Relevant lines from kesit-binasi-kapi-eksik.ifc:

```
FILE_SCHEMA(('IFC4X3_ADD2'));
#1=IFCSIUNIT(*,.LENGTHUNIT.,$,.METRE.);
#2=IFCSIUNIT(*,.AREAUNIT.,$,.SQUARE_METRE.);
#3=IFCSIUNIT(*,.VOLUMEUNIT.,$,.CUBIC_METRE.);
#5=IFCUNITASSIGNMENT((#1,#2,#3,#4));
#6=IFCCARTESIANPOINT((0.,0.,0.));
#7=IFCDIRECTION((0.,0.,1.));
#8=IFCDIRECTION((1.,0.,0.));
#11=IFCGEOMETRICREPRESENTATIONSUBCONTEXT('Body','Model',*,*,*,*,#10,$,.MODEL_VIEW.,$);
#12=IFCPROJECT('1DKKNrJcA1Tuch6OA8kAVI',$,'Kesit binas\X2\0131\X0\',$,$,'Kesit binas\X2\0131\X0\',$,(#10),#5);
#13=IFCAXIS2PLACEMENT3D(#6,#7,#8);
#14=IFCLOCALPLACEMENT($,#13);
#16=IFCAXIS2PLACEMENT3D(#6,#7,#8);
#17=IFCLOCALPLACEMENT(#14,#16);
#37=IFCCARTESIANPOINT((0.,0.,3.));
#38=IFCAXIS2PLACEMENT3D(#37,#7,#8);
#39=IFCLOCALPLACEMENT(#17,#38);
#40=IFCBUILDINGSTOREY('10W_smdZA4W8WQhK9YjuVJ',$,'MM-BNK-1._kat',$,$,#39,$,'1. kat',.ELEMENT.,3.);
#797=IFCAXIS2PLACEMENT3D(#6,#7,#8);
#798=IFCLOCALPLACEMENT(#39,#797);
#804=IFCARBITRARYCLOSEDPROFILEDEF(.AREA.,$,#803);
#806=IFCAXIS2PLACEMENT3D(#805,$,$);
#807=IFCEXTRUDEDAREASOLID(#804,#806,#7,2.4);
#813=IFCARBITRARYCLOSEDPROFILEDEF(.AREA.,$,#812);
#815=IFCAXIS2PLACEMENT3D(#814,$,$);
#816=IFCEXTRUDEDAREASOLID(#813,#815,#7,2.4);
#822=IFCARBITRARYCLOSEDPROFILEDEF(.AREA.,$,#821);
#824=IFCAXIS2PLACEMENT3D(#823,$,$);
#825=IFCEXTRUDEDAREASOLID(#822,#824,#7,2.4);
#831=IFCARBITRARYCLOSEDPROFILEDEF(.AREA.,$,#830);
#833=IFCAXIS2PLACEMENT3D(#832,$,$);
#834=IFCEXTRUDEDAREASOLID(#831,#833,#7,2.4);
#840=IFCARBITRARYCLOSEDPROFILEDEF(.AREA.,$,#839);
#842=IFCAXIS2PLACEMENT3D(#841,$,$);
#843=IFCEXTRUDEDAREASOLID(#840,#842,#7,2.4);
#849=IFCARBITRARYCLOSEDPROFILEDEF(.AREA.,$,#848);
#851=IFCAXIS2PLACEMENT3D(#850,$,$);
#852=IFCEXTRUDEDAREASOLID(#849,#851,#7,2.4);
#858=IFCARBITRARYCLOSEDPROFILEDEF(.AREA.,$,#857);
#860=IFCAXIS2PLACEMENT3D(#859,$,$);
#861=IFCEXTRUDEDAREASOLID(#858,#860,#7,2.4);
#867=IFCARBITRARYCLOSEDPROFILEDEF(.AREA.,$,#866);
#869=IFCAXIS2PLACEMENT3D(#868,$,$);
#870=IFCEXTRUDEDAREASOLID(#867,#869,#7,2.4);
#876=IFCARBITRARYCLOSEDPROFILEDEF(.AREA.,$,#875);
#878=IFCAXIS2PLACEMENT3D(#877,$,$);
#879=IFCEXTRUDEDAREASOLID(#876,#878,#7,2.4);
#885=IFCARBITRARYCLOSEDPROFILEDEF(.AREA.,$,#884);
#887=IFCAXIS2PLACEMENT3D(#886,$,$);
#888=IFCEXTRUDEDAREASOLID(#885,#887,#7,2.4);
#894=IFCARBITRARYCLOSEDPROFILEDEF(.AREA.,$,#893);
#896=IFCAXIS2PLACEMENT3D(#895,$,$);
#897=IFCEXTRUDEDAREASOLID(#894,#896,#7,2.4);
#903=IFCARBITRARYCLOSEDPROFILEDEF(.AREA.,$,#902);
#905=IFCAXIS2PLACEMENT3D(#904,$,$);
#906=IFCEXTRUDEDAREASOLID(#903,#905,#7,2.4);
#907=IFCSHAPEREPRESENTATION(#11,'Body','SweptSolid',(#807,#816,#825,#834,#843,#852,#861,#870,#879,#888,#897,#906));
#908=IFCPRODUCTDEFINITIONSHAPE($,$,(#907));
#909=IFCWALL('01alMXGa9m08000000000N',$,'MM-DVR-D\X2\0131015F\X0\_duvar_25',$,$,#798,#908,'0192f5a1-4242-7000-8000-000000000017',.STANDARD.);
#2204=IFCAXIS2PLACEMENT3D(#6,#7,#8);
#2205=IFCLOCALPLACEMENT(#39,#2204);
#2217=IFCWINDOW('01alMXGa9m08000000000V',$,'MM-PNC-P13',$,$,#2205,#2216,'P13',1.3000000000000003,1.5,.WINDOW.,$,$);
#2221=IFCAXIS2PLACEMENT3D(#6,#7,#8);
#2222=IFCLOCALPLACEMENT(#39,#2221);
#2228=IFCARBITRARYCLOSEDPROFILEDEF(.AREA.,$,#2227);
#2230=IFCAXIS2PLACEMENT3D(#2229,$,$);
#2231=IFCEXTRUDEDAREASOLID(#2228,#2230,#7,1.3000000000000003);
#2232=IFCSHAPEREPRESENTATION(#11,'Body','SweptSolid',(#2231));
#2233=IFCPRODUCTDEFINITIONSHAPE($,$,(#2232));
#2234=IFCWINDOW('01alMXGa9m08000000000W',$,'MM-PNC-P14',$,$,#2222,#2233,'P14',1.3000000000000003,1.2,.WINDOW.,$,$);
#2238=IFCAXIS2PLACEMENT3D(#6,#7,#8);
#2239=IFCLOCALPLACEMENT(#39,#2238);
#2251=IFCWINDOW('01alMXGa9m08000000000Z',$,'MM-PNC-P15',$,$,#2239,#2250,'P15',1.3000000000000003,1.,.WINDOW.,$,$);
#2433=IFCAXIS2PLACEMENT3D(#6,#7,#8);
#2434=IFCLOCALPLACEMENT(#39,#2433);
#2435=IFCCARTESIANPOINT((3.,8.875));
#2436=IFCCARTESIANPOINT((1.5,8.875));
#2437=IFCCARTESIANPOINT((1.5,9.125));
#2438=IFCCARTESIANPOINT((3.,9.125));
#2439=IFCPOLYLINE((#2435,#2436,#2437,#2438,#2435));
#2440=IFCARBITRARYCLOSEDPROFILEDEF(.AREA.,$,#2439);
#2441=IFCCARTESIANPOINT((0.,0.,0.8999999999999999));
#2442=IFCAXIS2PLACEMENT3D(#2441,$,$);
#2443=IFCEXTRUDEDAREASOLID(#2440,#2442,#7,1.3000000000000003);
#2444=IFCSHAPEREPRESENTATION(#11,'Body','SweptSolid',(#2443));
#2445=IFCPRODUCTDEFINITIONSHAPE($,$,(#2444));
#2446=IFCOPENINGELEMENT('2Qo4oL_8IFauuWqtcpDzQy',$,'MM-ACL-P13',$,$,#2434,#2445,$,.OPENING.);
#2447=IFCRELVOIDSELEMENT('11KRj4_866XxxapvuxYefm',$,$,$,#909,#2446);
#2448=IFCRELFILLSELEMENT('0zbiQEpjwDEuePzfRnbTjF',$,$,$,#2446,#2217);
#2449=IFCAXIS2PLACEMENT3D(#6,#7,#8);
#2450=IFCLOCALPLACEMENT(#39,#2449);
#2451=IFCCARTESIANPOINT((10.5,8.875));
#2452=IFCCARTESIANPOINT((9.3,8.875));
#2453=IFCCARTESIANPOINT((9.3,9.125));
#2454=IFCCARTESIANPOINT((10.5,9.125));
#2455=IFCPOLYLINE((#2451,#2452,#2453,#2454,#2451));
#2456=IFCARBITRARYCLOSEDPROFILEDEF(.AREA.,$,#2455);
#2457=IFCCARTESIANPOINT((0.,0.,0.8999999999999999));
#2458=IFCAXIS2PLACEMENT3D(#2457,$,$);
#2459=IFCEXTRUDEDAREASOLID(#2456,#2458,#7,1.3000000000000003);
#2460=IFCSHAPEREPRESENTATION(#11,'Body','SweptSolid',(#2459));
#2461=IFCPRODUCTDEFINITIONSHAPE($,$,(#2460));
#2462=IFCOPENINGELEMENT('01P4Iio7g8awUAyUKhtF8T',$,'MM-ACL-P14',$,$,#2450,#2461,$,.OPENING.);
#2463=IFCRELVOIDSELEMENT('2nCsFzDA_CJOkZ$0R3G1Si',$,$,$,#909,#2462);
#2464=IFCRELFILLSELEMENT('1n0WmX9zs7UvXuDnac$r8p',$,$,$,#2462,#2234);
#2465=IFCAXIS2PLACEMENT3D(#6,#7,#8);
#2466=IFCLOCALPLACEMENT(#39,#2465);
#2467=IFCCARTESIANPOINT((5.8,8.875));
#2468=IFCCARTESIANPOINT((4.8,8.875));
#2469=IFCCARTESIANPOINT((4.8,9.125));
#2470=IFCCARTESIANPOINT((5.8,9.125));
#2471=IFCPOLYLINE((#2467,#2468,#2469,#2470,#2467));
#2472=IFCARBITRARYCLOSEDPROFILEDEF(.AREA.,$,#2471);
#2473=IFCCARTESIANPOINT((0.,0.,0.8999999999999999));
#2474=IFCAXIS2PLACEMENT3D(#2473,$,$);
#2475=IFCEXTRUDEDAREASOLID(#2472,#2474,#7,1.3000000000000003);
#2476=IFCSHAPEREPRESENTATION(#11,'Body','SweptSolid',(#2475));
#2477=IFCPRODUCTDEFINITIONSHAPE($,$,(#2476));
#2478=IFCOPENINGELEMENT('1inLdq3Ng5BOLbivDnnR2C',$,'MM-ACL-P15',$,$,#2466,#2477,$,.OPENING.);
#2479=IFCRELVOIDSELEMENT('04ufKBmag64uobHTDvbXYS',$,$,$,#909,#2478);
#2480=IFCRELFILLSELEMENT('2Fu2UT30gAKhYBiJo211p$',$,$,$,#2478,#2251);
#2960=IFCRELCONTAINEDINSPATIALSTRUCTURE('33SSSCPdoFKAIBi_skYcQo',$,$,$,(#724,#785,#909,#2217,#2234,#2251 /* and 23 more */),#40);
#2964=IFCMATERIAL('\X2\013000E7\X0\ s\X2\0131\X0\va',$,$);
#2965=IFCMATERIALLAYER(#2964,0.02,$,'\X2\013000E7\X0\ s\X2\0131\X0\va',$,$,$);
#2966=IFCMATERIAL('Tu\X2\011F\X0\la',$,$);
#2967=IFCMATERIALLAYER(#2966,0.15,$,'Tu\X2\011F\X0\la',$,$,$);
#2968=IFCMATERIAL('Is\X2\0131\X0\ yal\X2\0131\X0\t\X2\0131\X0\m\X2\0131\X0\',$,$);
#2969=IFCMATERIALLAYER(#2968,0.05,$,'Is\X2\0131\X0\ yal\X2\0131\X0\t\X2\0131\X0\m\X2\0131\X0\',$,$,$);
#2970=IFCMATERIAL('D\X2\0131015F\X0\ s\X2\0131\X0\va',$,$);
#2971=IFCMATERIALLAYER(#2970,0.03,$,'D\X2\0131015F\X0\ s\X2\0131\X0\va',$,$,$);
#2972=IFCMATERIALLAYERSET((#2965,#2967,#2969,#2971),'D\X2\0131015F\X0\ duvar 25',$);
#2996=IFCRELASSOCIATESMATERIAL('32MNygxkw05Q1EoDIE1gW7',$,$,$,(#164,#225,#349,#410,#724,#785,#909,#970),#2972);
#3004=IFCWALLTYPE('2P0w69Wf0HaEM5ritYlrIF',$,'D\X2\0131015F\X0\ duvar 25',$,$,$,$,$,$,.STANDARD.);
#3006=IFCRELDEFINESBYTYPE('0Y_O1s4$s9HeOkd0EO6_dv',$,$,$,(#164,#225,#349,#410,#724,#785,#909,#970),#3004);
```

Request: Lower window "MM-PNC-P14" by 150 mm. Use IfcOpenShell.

```python
import numpy as np
import ifcopenshell
import ifcopenshell.api.geometry
import ifcopenshell.util.placement
import ifcopenshell.util.unit

model = ifcopenshell.open("kesit-binasi-kapi-eksik.ifc")
unit_scale = ifcopenshell.util.unit.calculate_unit_scale(model)

window = model.by_id(2234)
opening = window.FillsVoids[0].RelatingOpeningElement
dz = -0.15 / unit_scale

shift = np.array([0.0, 0.0, dz])
# The window is not placed relative to its opening, so move both.
for product in (opening, window):
    matrix = ifcopenshell.util.placement.get_local_placement(product.ObjectPlacement)
    matrix[:3, 3] += shift
    ifcopenshell.api.geometry.edit_object_placement(model, product=product, matrix=matrix, is_si=False)

print(f"moved by {dz * unit_scale:+.3f} m")

model.write("kesit-binasi-kapi-eksik_edited.ifc")
```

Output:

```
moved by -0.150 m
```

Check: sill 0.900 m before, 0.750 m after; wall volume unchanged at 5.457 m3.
